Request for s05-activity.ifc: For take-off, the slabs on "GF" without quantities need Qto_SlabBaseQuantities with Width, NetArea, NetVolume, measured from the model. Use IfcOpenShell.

First a look at what the model holds.

```python
import ifcopenshell
import ifcopenshell.util.element
import ifcopenshell.util.unit

model = ifcopenshell.open("s05-activity.ifc")
print(model.schema)
for unit_type in ("LENGTHUNIT", "AREAUNIT", "VOLUMEUNIT"):
    print(unit_type, ifcopenshell.util.unit.calculate_unit_scale(model, unit_type))
storey = next(s for s in model.by_type("IfcBuildingStorey") if s.Name == "GF")
slabs = [e for e in ifcopenshell.util.element.get_decomposition(storey) if e.is_a("IfcSlab")]
for e in sorted(slabs, key=lambda e: e.id()):
    print(e.id(), e.is_a(), e.Name, list(ifcopenshell.util.element.get_psets(e, qtos_only=True)), sep=" | ")
```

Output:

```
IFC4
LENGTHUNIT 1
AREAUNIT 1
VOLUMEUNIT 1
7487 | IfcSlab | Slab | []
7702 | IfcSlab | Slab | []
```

```python
import ifcopenshell
import ifcopenshell.api.pset
import ifcopenshell.geom
import ifcopenshell.util.element
import ifcopenshell.util.shape
import ifcopenshell.util.unit

model = ifcopenshell.open("s05-activity.ifc")
unit_scale = ifcopenshell.util.unit.calculate_unit_scale(model)
area_scale = ifcopenshell.util.unit.calculate_unit_scale(model, "AREAUNIT")
volume_scale = ifcopenshell.util.unit.calculate_unit_scale(model, "VOLUMEUNIT")
settings = ifcopenshell.geom.settings()

storey = next(s for s in model.by_type("IfcBuildingStorey") if s.Name == "GF")
slabs = [e for e in ifcopenshell.util.element.get_decomposition(storey) if e.is_a("IfcSlab")]

for e in sorted(slabs, key=lambda e: e.id()):
    if ifcopenshell.util.element.get_psets(e, qtos_only=True, should_inherit=False):
        continue
    # Geometry comes back in metres, in the element's own axes.
    shape = ifcopenshell.geom.create_shape(settings, e)
    values = {
        "Width": ifcopenshell.util.shape.get_z(shape.geometry) / unit_scale,
        "NetArea": ifcopenshell.util.shape.get_footprint_area(shape.geometry) / area_scale,
        "NetVolume": ifcopenshell.util.shape.get_volume(shape.geometry) / volume_scale,
    }
    qto = ifcopenshell.api.pset.add_qto(model, product=e, name="Qto_SlabBaseQuantities")
    ifcopenshell.api.pset.edit_qto(model, qto=qto, properties=values)
    print(e.id(), {k: round(v, 3) for k, v in values.items()})

model.write("s05-activity_updated.ifc")
```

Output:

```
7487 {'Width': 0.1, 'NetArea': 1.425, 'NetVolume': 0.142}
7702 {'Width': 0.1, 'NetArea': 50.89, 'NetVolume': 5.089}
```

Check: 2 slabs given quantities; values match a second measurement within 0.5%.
